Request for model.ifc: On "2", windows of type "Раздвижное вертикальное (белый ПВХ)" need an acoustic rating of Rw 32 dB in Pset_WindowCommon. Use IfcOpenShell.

First a look at what the model holds.

```python
import ifcopenshell
import ifcopenshell.util.element

model = ifcopenshell.open("model.ifc")
print(model.schema)
storey = next(s for s in model.by_type("IfcBuildingStorey") if s.Name == "2")
windows = [e for e in ifcopenshell.util.element.get_decomposition(storey) if e.is_a("IfcWindow")]
seen = {}
for e in windows:
    element_type = ifcopenshell.util.element.get_type(e)
    key = (element_type.Name if element_type != e and element_type else None, ifcopenshell.util.element.get_pset(e, "Pset_WindowCommon", "AcousticRating"))
    seen[key] = seen.get(key, 0) + 1
for (name, value), count in sorted(seen.items(), key=str):
    print(count, "x", name, "|", value)
```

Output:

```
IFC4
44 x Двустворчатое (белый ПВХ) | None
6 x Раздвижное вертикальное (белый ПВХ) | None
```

```python
import ifcopenshell
import ifcopenshell.api.pset
import ifcopenshell.util.element

model = ifcopenshell.open("model.ifc")

storey = next(s for s in model.by_type("IfcBuildingStorey") if s.Name == "2")
windows = [e for e in ifcopenshell.util.element.get_decomposition(storey) if e.is_a("IfcWindow")]

count = 0
for e in windows:
    element_type = ifcopenshell.util.element.get_type(e)
    if element_type in (None, e) or element_type.Name != "Раздвижное вертикальное (белый ПВХ)":
        continue
    # add_pset returns the element's existing set when there is one.
    pset = ifcopenshell.api.pset.add_pset(model, product=e, name="Pset_WindowCommon")
    ifcopenshell.api.pset.edit_pset(model, pset=pset, properties={"AcousticRating": "Rw 32 dB"})
    count += 1

print(count, "windows updated")

model.write("model_v2.ifc")
```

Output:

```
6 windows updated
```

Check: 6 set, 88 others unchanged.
